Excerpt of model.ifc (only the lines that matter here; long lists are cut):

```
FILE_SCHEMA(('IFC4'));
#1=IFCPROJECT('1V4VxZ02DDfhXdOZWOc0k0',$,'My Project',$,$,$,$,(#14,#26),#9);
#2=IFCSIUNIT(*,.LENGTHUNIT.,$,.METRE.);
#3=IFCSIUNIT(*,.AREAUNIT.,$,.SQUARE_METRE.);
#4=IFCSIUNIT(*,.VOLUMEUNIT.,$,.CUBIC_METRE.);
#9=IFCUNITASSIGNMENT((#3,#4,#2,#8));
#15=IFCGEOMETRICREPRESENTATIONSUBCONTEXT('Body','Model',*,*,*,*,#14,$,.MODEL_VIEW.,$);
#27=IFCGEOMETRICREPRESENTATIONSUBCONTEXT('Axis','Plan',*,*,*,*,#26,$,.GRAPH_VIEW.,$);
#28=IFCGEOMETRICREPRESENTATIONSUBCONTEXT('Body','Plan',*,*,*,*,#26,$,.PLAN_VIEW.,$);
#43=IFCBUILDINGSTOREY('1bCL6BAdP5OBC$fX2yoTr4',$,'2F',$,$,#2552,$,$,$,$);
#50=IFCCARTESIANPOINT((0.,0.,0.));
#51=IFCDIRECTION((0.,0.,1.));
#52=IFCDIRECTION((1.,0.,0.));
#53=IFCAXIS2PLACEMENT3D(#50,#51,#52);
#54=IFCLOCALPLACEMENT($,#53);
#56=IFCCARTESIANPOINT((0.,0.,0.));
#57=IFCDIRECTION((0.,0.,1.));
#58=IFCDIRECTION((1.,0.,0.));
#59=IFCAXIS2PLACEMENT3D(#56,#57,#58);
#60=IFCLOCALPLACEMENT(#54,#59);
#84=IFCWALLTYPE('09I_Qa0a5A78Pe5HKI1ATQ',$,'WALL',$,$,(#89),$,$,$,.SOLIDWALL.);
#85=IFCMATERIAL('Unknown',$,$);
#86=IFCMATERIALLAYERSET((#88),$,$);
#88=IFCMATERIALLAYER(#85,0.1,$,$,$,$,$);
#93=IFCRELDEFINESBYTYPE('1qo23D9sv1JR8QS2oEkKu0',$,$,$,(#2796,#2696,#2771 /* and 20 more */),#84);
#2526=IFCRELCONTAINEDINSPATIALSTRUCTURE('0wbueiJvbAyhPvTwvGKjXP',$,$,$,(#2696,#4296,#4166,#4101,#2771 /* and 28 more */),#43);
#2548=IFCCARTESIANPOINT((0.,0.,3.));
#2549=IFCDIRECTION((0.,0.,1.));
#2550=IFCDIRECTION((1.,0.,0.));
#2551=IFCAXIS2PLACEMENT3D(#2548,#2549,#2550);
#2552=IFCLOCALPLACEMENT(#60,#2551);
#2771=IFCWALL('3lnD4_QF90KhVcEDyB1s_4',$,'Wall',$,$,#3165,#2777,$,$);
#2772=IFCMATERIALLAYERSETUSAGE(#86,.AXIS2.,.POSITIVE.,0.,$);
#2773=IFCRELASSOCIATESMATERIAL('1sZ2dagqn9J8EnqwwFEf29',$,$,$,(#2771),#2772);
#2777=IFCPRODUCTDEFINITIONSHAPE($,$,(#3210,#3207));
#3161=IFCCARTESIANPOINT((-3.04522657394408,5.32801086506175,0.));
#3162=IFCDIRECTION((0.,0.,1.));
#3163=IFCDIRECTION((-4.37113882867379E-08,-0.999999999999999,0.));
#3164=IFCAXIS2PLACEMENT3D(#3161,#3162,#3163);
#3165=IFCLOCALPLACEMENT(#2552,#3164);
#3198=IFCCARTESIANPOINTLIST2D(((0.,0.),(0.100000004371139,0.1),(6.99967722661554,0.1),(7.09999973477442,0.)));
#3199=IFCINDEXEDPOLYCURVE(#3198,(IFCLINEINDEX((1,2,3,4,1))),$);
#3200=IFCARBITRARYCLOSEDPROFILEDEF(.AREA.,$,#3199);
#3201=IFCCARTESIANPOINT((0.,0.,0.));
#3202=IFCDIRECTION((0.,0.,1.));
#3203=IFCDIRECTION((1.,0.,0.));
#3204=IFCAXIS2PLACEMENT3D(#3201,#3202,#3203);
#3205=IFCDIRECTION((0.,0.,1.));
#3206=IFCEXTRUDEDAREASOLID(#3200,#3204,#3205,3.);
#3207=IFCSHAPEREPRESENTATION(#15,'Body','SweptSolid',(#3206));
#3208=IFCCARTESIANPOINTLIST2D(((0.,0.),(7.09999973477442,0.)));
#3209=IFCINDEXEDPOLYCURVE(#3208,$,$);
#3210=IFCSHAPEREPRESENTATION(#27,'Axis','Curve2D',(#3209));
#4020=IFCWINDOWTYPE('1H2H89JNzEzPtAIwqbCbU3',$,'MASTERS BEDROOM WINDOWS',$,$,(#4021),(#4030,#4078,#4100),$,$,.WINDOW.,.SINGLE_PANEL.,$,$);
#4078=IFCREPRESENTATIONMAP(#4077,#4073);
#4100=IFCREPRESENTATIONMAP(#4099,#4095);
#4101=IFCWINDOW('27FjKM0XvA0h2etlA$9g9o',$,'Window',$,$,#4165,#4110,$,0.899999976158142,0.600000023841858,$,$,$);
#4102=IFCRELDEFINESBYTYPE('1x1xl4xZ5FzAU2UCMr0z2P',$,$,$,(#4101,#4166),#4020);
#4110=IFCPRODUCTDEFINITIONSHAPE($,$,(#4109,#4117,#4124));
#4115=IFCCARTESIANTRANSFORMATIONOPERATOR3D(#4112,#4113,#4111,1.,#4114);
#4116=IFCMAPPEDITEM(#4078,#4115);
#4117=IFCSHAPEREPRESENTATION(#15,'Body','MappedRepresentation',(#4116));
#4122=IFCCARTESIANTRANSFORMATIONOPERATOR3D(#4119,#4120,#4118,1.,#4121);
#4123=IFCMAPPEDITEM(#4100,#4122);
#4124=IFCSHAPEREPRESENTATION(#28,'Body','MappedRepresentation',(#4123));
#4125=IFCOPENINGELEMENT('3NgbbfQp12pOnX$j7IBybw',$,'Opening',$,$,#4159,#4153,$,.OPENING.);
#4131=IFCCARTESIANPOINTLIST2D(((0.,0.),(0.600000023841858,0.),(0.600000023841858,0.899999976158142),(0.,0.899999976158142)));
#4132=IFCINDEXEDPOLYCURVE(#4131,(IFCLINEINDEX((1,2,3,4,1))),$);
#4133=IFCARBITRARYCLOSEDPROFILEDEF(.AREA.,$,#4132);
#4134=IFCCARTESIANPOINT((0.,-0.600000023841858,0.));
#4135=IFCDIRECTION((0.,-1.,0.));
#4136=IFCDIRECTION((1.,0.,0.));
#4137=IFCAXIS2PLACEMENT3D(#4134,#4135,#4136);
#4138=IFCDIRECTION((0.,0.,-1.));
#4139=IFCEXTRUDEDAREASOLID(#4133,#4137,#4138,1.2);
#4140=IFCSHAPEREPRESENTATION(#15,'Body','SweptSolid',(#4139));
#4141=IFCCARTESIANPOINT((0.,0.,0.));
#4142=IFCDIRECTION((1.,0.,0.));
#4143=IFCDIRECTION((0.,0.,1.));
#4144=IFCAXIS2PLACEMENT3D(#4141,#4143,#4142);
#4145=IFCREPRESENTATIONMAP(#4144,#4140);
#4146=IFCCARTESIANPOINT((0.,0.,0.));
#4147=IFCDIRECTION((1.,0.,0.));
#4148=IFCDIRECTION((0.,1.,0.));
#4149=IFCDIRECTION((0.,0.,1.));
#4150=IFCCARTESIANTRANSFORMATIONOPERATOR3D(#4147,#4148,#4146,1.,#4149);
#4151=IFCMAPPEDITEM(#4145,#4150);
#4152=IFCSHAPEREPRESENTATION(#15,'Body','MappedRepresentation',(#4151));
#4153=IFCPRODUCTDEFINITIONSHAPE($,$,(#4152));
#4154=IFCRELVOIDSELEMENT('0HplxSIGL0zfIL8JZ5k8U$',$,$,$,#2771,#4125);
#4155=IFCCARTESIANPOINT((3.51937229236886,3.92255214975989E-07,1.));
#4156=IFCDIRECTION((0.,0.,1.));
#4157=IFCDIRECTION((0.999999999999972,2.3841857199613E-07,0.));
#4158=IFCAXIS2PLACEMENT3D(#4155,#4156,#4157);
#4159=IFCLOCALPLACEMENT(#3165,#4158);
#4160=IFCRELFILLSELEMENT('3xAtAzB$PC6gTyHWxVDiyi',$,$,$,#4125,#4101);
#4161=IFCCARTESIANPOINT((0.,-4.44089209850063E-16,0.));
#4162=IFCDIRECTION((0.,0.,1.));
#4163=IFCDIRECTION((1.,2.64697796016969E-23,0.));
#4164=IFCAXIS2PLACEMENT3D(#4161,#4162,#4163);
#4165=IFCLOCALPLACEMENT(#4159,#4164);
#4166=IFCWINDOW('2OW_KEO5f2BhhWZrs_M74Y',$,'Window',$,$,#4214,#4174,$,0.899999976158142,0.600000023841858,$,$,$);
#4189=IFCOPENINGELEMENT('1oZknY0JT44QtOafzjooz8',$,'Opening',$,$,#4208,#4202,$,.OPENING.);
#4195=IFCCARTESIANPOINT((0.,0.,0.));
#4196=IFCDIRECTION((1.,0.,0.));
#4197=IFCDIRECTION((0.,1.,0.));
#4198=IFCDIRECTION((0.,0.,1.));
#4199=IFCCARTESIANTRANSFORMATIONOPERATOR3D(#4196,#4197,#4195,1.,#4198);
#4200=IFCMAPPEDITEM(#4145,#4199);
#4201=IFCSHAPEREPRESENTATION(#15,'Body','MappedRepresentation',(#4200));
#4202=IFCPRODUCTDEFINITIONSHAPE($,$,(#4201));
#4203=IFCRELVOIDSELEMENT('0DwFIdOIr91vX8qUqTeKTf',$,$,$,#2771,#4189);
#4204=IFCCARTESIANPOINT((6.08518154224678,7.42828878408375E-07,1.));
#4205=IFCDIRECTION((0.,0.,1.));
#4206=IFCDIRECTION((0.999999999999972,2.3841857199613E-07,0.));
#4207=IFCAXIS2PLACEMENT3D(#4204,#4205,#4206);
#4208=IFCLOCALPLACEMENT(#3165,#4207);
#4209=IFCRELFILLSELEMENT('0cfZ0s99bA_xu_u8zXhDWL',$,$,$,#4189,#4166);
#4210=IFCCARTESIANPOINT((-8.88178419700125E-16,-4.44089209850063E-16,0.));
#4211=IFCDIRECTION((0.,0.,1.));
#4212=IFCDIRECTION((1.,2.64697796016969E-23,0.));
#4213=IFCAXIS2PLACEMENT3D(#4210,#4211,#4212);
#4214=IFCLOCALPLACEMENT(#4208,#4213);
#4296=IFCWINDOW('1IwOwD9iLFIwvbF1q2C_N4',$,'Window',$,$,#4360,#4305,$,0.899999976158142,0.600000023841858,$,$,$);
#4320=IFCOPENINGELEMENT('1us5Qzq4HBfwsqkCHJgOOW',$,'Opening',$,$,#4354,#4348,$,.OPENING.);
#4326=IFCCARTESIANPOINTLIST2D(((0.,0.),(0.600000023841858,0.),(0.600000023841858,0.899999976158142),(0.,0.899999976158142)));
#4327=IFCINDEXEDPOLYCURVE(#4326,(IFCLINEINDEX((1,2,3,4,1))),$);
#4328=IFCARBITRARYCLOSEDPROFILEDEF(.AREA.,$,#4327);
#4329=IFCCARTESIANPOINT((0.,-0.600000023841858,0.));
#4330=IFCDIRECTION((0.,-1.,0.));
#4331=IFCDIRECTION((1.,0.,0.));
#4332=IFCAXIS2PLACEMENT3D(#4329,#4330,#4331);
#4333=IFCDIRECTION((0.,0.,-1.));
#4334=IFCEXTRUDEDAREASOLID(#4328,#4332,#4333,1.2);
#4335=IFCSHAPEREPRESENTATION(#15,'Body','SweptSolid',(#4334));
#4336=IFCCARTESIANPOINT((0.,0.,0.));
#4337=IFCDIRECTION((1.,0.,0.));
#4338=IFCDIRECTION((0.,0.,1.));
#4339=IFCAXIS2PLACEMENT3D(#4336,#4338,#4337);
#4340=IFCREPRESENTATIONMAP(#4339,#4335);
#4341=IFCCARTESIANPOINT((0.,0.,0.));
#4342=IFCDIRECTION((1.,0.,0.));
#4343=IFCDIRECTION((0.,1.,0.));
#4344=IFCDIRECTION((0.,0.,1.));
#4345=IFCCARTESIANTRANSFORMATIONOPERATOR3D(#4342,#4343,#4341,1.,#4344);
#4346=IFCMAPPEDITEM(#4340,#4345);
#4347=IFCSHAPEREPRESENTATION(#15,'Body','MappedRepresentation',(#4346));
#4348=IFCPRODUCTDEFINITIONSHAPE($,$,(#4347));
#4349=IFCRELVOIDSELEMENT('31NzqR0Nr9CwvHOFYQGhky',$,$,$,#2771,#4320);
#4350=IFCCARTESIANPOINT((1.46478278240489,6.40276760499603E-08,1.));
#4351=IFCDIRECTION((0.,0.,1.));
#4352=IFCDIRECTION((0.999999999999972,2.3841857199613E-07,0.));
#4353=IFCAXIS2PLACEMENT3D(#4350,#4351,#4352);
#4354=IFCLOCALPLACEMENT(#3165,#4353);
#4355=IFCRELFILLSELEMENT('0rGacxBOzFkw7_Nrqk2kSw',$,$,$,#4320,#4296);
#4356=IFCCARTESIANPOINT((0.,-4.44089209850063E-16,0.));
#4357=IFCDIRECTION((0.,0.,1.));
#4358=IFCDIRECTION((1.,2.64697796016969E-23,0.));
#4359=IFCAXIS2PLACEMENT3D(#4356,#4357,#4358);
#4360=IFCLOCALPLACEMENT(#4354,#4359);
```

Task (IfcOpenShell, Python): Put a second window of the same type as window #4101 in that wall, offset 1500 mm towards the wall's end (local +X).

```python
import ifcopenshell
import ifcopenshell.api.feature
import ifcopenshell.api.geometry
import ifcopenshell.api.root
import ifcopenshell.geom
import ifcopenshell.util.element
import ifcopenshell.util.placement
import ifcopenshell.util.shape
import ifcopenshell.util.unit

model = ifcopenshell.open("model.ifc")
unit_scale = ifcopenshell.util.unit.calculate_unit_scale(model)
settings = ifcopenshell.geom.settings()


def volume(element):
    """Net volume in cubic metres, openings subtracted."""
    shape = ifcopenshell.geom.create_shape(settings, element)
    return ifcopenshell.util.shape.get_volume(shape.geometry)


window = model.by_guid("27FjKM0XvA0h2etlA$9g9o")
opening = window.FillsVoids[0].RelatingOpeningElement
wall = opening.VoidsElements[0].RelatingBuildingElement
before = volume(wall)
shift = ifcopenshell.util.placement.get_local_placement(wall.ObjectPlacement)[:3, 0] * 1.5 / unit_scale

# copy_class copies the void relationship, type, container and properties, but no geometry.
new_opening = ifcopenshell.api.root.copy_class(model, product=opening)
new_opening.Representation = ifcopenshell.util.element.copy_deep(
    model, opening.Representation, exclude=["IfcGeometricRepresentationContext", "IfcRepresentationMap"]
)
new_window = ifcopenshell.api.root.copy_class(model, product=window)
new_window.Representation = ifcopenshell.util.element.copy_deep(
    model, window.Representation, exclude=["IfcGeometricRepresentationContext", "IfcRepresentationMap"]
)
ifcopenshell.api.feature.add_filling(model, opening=new_opening, element=new_window)

for old, new in ((opening, new_opening), (window, new_window)):
    matrix = ifcopenshell.util.placement.get_local_placement(old.ObjectPlacement)
    matrix[:3, 3] += shift
    ifcopenshell.api.geometry.edit_object_placement(model, product=new, matrix=matrix, is_si=False)

after = volume(wall)

print(f"wall volume {before:.3f} -> {after:.3f} m3")

model.write("model_rev.ifc")
```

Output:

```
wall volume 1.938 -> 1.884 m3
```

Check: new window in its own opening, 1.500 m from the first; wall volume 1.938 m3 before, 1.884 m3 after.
